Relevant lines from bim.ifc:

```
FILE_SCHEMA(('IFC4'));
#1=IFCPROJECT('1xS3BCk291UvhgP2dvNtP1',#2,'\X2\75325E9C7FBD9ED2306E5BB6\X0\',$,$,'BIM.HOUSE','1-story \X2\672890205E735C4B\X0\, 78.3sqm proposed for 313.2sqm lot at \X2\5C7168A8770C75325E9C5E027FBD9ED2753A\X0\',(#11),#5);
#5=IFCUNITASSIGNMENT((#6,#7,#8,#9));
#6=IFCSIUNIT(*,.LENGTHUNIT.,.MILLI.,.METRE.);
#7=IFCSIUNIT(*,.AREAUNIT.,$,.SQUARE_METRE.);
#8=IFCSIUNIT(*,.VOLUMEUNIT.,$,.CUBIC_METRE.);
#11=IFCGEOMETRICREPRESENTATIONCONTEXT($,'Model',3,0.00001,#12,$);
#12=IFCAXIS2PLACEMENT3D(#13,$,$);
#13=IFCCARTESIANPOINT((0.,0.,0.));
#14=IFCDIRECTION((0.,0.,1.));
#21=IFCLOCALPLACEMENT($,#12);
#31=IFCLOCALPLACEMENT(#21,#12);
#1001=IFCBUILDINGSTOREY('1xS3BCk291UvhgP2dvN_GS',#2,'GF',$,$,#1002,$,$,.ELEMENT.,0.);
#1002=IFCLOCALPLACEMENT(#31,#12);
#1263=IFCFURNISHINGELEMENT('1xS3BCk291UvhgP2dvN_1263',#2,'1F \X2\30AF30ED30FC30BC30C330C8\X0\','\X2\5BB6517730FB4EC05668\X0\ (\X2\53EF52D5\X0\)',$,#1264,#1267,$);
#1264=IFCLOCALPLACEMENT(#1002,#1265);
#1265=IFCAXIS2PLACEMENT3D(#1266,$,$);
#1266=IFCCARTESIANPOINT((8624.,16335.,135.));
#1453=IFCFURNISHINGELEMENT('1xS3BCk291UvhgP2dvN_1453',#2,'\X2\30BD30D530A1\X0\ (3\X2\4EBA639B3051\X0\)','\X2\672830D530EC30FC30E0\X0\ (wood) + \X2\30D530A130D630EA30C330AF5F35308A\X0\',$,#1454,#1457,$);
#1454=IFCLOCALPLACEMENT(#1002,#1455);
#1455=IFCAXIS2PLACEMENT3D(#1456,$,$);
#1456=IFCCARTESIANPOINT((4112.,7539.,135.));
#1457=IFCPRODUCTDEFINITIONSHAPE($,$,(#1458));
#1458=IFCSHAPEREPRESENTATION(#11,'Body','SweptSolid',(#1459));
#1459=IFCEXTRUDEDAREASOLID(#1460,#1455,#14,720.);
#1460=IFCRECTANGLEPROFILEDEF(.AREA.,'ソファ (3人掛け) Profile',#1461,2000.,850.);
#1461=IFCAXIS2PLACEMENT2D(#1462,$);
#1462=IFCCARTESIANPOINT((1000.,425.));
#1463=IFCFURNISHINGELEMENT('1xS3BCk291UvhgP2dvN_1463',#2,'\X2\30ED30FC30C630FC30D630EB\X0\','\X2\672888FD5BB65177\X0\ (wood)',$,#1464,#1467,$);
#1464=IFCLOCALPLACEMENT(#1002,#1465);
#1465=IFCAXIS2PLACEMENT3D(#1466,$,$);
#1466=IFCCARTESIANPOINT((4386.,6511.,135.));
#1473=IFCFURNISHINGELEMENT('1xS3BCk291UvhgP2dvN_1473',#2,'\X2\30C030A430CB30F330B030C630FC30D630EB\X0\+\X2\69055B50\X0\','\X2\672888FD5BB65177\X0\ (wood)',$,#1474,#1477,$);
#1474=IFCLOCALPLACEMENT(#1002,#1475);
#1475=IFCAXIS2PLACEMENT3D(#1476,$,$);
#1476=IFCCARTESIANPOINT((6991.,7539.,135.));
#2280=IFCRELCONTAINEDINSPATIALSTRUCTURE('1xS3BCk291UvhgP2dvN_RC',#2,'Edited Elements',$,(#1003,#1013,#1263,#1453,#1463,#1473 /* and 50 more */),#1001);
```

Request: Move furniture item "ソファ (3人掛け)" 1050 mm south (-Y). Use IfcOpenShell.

```python
import ifcopenshell
import ifcopenshell.api.geometry
import ifcopenshell.util.placement

model = ifcopenshell.open("bim.ifc")

item = model.by_guid("1xS3BCk291UvhgP2dvN_1453")
matrix = ifcopenshell.util.placement.get_local_placement(item.ObjectPlacement)
matrix[1, 3] -= 1050.0
ifcopenshell.api.geometry.edit_object_placement(model, product=item, matrix=matrix, is_si=False)

print(ifcopenshell.util.placement.get_local_placement(item.ObjectPlacement).round(3) + 0.0)

model.write("bim_v2.ifc")
```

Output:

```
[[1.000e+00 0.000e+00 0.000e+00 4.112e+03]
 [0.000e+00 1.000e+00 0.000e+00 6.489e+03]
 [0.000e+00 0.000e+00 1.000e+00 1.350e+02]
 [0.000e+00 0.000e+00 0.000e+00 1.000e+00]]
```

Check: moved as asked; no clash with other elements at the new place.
